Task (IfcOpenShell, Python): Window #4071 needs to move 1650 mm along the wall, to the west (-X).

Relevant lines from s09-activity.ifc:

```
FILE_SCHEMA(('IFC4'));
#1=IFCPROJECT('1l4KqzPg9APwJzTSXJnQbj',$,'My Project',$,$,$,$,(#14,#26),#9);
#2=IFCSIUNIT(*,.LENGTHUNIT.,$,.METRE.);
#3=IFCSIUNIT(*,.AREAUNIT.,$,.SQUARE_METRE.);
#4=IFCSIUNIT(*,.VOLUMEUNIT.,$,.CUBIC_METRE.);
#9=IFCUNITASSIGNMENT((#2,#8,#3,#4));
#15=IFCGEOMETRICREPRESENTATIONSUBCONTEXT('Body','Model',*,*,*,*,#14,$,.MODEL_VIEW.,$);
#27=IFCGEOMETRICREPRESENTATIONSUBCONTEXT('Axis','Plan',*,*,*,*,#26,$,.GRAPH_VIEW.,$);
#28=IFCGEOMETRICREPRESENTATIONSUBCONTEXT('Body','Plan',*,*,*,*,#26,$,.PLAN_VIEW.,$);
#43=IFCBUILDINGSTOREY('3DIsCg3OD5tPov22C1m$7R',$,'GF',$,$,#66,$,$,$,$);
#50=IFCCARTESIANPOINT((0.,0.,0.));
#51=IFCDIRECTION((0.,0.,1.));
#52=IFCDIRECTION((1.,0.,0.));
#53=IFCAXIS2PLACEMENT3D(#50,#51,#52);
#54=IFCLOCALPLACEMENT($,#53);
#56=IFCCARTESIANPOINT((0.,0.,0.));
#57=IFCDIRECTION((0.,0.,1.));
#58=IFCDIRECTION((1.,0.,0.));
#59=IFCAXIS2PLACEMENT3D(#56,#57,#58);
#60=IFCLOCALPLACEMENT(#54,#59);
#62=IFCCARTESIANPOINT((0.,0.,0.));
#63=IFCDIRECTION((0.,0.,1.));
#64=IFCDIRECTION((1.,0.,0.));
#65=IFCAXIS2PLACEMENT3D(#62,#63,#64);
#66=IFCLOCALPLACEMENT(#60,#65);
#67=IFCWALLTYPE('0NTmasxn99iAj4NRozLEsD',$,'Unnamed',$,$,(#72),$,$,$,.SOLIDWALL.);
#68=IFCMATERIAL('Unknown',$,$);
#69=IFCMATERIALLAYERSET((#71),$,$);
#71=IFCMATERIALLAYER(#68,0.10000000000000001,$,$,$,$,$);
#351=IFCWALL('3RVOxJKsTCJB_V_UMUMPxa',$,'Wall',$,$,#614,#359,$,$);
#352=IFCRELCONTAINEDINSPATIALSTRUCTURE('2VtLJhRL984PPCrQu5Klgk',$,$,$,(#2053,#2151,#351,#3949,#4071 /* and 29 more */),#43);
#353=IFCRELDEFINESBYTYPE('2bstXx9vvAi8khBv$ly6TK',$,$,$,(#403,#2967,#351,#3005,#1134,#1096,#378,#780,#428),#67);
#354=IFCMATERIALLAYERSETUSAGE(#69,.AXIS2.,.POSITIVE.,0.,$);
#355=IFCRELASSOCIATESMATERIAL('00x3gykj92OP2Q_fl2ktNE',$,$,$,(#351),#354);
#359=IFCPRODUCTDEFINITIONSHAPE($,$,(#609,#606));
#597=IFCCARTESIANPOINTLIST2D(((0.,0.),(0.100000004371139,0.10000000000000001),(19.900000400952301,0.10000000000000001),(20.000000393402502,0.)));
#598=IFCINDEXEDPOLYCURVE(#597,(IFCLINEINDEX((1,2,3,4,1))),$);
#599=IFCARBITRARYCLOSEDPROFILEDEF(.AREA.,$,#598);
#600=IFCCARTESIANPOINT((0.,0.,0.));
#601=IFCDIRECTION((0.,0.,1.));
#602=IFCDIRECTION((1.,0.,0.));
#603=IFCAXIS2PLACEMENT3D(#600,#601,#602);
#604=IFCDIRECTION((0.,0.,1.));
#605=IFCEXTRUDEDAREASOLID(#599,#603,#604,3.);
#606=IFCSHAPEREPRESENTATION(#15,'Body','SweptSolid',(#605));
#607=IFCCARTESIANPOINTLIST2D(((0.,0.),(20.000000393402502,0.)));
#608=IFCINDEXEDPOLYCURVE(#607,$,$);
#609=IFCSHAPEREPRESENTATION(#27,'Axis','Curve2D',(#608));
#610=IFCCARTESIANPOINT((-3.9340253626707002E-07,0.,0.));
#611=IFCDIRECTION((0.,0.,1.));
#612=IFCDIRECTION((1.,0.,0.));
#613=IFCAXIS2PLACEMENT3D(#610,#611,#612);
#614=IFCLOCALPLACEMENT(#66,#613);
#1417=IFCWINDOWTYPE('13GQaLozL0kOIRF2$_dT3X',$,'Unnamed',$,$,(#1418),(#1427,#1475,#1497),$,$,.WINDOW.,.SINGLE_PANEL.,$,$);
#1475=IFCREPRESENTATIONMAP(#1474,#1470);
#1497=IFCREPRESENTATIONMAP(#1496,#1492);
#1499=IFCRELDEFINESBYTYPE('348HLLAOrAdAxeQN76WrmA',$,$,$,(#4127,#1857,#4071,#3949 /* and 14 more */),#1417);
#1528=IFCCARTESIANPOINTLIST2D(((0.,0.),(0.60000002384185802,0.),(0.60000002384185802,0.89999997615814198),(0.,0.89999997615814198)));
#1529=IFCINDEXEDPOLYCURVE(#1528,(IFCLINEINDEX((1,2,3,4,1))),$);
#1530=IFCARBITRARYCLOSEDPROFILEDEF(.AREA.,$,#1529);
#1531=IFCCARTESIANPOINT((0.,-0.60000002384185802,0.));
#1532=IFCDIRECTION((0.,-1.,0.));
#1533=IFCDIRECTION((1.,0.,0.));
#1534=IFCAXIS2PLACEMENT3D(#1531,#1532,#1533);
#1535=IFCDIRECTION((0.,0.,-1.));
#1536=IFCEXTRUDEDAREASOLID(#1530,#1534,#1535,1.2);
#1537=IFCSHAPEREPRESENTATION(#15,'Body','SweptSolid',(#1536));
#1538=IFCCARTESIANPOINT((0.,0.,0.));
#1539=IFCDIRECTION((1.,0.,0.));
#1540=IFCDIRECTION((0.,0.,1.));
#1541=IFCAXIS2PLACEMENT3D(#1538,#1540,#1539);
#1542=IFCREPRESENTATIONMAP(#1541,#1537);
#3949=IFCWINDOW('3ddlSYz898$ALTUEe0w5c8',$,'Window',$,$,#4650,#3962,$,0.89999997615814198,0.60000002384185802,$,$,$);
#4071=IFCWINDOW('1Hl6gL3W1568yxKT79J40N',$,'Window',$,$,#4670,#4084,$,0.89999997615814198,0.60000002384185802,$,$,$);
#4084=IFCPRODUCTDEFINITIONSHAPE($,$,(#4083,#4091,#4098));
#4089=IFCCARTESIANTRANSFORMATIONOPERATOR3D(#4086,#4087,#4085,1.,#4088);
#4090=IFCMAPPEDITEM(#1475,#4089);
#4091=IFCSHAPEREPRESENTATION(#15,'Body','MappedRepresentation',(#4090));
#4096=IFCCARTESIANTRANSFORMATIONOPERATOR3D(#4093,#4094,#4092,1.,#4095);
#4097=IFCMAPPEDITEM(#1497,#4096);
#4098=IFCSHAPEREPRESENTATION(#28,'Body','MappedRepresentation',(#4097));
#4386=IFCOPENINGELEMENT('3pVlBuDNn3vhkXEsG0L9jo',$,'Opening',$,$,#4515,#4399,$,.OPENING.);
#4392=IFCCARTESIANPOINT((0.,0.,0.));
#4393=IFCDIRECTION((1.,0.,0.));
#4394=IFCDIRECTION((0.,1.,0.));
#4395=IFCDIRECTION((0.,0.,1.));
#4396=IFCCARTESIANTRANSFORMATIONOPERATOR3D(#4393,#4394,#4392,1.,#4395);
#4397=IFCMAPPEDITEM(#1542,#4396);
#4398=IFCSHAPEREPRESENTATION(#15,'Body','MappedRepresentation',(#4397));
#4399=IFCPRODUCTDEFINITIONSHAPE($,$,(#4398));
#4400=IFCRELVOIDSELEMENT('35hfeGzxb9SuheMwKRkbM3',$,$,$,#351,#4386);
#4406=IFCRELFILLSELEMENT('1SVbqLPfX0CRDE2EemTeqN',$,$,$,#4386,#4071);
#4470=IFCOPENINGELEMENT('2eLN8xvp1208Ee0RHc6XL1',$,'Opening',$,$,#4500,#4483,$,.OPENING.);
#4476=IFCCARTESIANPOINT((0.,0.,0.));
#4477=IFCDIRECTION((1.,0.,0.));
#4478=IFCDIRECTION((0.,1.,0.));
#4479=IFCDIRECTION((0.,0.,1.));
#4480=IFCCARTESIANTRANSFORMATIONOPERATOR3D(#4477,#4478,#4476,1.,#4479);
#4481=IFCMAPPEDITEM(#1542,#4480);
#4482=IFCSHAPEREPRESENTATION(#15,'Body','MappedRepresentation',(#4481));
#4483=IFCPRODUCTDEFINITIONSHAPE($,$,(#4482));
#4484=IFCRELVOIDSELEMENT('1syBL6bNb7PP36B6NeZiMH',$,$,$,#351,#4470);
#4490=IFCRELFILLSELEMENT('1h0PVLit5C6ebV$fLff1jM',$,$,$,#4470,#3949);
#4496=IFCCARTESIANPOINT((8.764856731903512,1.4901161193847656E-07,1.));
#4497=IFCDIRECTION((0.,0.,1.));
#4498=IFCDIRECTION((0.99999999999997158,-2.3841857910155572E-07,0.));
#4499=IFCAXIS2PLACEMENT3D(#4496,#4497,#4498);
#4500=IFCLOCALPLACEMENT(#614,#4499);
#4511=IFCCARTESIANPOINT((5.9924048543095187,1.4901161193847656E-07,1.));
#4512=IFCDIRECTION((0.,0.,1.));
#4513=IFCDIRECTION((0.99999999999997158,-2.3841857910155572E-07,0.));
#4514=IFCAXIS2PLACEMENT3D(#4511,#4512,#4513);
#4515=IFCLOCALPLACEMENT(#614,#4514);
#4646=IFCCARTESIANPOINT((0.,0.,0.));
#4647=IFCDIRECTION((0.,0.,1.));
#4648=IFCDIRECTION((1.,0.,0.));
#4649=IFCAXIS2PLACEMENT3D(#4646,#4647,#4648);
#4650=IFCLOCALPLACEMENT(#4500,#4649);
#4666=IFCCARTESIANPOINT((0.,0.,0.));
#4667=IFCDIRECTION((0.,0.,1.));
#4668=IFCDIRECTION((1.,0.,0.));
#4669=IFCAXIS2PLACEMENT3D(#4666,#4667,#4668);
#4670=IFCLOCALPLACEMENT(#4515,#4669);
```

```python
import ifcopenshell
import ifcopenshell.api.geometry
import ifcopenshell.util.placement

model = ifcopenshell.open("s09-activity.ifc")

window = model.by_guid("1Hl6gL3W1568yxKT79J40N")
opening = window.FillsVoids[0].RelatingOpeningElement
wall = opening.VoidsElements[0].RelatingBuildingElement

wall_matrix = ifcopenshell.util.placement.get_local_placement(wall.ObjectPlacement)
shift = wall_matrix[:3, 0] * -1.65
before = ifcopenshell.util.placement.get_local_placement(window.ObjectPlacement)[:3, 3].copy()

# The window is placed relative to its opening, so it follows when the opening moves.
matrix = ifcopenshell.util.placement.get_local_placement(opening.ObjectPlacement)
matrix[:3, 3] += shift
ifcopenshell.api.geometry.edit_object_placement(
    model, product=opening, matrix=matrix, is_si=False, should_transform_children=True
)

after = ifcopenshell.util.placement.get_local_placement(window.ObjectPlacement)[:3, 3]
print("window moved by", (after - before).round(3) + 0.0)

model.write("s09-activity_updated.ifc")
```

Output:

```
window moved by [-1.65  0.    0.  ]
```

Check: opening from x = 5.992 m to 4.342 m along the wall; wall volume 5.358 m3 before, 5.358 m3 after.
